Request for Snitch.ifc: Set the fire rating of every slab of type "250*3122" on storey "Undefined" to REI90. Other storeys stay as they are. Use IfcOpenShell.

First a look at what the model holds.

```python
import ifcopenshell
import ifcopenshell.util.element

model = ifcopenshell.open("Snitch.ifc")
print(model.schema)
storey = next(s for s in model.by_type("IfcBuildingStorey") if s.Name == "Undefined")
slabs = [e for e in ifcopenshell.util.element.get_decomposition(storey) if e.is_a("IfcSlab")]
seen = {}
for e in slabs:
    element_type = ifcopenshell.util.element.get_type(e)
    key = (element_type.Name if element_type != e and element_type else None, ifcopenshell.util.element.get_pset(e, "Pset_SlabCommon", "FireRating"))
    seen[key] = seen.get(key, 0) + 1
for (name, value), count in sorted(seen.items(), key=str):
    print(count, "x", name, "|", value)
```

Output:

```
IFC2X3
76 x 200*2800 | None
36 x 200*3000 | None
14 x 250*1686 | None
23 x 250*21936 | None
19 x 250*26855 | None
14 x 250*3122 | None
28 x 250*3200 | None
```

```python
import ifcopenshell
import ifcopenshell.api.pset
import ifcopenshell.util.element

model = ifcopenshell.open("Snitch.ifc")

storey = next(s for s in model.by_type("IfcBuildingStorey") if s.Name == "Undefined")
slabs = [e for e in ifcopenshell.util.element.get_decomposition(storey) if e.is_a("IfcSlab")]

count = 0
for e in slabs:
    element_type = ifcopenshell.util.element.get_type(e)
    if element_type in (None, e) or element_type.Name != "250*3122":
        continue
    found = ifcopenshell.util.element.get_pset(e, "Pset_SlabCommon", should_inherit=False)
    if found:
        pset = model.by_id(found["id"])
        if len(ifcopenshell.util.element.get_elements_by_pset(pset)) > 1:
            pset = ifcopenshell.api.pset.unshare_pset(model, products=[e], pset=pset)[0]
    else:
        pset = ifcopenshell.api.pset.add_pset(model, product=e, name="Pset_SlabCommon")
    ifcopenshell.api.pset.edit_pset(model, pset=pset, properties={"FireRating": "REI90"})
    count += 1

print(count, "slabs updated")

model.write("Snitch_v2.ifc")
```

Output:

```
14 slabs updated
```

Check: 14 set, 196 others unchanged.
